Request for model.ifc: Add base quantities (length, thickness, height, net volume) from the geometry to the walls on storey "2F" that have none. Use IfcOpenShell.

First a look at what the model holds.

```python
import ifcopenshell
import ifcopenshell.util.element
import ifcopenshell.util.unit

model = ifcopenshell.open("model.ifc")
print(model.schema)
for unit_type in ("LENGTHUNIT", "AREAUNIT", "VOLUMEUNIT"):
    print(unit_type, ifcopenshell.util.unit.calculate_unit_scale(model, unit_type))
storey = next(s for s in model.by_type("IfcBuildingStorey") if s.Name == "2F")
walls = [e for e in ifcopenshell.util.element.get_decomposition(storey) if e.is_a("IfcWall")]
for e in sorted(walls, key=lambda e: e.id()):
    print(e.id(), e.is_a(), e.Name, list(ifcopenshell.util.element.get_psets(e, qtos_only=True)), sep=" | ")
```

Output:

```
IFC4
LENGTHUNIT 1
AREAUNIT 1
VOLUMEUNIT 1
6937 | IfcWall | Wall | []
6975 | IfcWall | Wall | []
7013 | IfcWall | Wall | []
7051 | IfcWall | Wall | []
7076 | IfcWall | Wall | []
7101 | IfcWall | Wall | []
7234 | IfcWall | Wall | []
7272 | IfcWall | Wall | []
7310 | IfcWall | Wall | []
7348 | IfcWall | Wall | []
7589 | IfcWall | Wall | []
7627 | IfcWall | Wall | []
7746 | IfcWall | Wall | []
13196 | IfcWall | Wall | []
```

```python
import ifcopenshell
import ifcopenshell.api.pset
import ifcopenshell.geom
import ifcopenshell.util.element
import ifcopenshell.util.shape
import ifcopenshell.util.unit

model = ifcopenshell.open("model.ifc")
unit_scale = ifcopenshell.util.unit.calculate_unit_scale(model)
volume_scale = ifcopenshell.util.unit.calculate_unit_scale(model, "VOLUMEUNIT")
settings = ifcopenshell.geom.settings()

storey = next(s for s in model.by_type("IfcBuildingStorey") if s.Name == "2F")
walls = [e for e in ifcopenshell.util.element.get_decomposition(storey) if e.is_a("IfcWall")]

for e in sorted(walls, key=lambda e: e.id()):
    if ifcopenshell.util.element.get_psets(e, qtos_only=True, should_inherit=False):
        continue
    # Geometry comes back in metres, in the element's own axes.
    shape = ifcopenshell.geom.create_shape(settings, e)
    values = {
        "Length": ifcopenshell.util.shape.get_x(shape.geometry) / unit_scale,
        "Width": ifcopenshell.util.shape.get_y(shape.geometry) / unit_scale,
        "Height": ifcopenshell.util.shape.get_z(shape.geometry) / unit_scale,
        "NetVolume": ifcopenshell.util.shape.get_volume(shape.geometry) / volume_scale,
    }
    qto = ifcopenshell.api.pset.add_qto(model, product=e, name="Qto_WallBaseQuantities")
    ifcopenshell.api.pset.edit_qto(model, qto=qto, properties=values)
    print(e.id(), {k: round(v, 3) for k, v in values.items()})

model.write("model-out.ifc")
```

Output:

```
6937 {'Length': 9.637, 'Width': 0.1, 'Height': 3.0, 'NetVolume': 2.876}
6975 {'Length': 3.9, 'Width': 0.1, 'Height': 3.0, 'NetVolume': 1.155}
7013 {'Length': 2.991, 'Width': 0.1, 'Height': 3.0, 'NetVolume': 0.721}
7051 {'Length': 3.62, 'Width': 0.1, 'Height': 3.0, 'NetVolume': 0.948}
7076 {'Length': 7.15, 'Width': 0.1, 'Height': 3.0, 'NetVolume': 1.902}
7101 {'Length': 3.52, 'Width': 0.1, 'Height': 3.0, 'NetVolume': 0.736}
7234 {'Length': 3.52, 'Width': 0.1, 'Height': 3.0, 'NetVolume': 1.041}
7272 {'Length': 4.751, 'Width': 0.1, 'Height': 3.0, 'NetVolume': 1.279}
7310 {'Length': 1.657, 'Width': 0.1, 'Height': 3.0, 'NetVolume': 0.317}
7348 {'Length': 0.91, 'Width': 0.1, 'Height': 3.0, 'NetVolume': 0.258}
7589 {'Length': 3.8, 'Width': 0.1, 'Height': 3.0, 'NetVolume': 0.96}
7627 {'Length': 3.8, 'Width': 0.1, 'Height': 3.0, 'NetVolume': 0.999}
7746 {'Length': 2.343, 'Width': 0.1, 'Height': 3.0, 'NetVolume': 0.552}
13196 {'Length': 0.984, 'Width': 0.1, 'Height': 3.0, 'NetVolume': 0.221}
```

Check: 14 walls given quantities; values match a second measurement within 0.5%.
